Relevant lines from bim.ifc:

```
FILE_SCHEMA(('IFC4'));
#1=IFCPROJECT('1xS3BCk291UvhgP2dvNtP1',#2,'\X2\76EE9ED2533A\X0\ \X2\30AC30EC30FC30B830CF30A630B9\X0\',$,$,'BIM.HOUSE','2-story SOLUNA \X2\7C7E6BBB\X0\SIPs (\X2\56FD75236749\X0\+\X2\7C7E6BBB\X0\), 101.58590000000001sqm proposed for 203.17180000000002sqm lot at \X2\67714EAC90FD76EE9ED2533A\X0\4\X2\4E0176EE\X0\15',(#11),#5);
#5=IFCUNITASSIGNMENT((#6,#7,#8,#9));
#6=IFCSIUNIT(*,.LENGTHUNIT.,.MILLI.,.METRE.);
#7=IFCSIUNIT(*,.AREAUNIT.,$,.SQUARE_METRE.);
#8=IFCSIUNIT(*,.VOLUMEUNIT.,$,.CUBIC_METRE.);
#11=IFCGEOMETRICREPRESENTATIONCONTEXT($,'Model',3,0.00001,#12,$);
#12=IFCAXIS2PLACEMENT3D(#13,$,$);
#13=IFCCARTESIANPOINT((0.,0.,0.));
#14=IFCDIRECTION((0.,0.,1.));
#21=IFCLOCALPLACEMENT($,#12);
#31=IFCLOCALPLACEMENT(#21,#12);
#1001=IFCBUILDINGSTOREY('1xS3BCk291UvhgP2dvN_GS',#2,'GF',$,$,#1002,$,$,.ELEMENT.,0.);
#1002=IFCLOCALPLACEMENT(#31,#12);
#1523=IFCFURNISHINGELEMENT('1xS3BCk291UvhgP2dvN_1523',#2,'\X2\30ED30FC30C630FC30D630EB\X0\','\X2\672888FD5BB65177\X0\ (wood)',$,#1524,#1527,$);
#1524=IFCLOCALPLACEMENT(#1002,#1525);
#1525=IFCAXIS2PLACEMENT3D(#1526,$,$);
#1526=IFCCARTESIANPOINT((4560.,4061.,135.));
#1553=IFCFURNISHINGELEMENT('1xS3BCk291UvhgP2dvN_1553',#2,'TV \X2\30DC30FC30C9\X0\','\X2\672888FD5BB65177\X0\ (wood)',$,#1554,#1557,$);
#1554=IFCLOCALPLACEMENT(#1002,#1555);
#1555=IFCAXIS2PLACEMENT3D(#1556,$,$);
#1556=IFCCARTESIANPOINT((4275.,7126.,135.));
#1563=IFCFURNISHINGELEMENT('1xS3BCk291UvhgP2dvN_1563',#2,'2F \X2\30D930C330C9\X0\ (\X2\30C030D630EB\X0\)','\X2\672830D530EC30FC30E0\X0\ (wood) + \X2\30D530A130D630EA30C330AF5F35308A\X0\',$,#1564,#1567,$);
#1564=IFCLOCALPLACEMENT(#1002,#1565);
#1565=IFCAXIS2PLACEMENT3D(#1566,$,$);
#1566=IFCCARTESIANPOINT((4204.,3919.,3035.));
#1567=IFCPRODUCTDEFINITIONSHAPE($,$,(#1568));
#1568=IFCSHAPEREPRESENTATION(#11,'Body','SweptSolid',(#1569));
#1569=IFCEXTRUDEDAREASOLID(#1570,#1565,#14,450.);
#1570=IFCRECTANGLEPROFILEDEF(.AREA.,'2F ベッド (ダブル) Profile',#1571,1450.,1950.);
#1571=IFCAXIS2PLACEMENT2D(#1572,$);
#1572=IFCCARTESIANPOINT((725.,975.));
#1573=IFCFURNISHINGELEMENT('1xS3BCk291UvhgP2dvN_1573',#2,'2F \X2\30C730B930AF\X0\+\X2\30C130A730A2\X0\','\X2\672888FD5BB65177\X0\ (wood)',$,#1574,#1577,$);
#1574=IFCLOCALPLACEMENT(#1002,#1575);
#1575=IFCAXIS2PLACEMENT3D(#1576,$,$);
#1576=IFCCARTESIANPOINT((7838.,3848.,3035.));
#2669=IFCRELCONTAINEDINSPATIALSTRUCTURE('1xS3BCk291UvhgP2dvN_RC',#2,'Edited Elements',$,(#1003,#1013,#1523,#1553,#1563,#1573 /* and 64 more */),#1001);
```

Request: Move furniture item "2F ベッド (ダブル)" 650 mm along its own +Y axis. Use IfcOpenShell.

```python
import ifcopenshell
import ifcopenshell.api.geometry
import ifcopenshell.util.placement
import ifcopenshell.util.unit

model = ifcopenshell.open("bim.ifc")
unit_scale = ifcopenshell.util.unit.calculate_unit_scale(model)

item = model.by_id(1563)
matrix = ifcopenshell.util.placement.get_local_placement(item.ObjectPlacement)
matrix[:3, 3] += matrix[:3, 1] * 0.65 / unit_scale
ifcopenshell.api.geometry.edit_object_placement(model, product=item, matrix=matrix, is_si=False)

print(ifcopenshell.util.placement.get_local_placement(item.ObjectPlacement).round(3) + 0.0)

model.write("bim_v2.ifc")
```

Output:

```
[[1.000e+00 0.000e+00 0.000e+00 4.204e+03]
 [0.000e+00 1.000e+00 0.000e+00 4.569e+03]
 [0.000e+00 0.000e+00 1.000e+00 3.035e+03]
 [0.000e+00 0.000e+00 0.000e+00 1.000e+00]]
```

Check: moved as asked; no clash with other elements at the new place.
